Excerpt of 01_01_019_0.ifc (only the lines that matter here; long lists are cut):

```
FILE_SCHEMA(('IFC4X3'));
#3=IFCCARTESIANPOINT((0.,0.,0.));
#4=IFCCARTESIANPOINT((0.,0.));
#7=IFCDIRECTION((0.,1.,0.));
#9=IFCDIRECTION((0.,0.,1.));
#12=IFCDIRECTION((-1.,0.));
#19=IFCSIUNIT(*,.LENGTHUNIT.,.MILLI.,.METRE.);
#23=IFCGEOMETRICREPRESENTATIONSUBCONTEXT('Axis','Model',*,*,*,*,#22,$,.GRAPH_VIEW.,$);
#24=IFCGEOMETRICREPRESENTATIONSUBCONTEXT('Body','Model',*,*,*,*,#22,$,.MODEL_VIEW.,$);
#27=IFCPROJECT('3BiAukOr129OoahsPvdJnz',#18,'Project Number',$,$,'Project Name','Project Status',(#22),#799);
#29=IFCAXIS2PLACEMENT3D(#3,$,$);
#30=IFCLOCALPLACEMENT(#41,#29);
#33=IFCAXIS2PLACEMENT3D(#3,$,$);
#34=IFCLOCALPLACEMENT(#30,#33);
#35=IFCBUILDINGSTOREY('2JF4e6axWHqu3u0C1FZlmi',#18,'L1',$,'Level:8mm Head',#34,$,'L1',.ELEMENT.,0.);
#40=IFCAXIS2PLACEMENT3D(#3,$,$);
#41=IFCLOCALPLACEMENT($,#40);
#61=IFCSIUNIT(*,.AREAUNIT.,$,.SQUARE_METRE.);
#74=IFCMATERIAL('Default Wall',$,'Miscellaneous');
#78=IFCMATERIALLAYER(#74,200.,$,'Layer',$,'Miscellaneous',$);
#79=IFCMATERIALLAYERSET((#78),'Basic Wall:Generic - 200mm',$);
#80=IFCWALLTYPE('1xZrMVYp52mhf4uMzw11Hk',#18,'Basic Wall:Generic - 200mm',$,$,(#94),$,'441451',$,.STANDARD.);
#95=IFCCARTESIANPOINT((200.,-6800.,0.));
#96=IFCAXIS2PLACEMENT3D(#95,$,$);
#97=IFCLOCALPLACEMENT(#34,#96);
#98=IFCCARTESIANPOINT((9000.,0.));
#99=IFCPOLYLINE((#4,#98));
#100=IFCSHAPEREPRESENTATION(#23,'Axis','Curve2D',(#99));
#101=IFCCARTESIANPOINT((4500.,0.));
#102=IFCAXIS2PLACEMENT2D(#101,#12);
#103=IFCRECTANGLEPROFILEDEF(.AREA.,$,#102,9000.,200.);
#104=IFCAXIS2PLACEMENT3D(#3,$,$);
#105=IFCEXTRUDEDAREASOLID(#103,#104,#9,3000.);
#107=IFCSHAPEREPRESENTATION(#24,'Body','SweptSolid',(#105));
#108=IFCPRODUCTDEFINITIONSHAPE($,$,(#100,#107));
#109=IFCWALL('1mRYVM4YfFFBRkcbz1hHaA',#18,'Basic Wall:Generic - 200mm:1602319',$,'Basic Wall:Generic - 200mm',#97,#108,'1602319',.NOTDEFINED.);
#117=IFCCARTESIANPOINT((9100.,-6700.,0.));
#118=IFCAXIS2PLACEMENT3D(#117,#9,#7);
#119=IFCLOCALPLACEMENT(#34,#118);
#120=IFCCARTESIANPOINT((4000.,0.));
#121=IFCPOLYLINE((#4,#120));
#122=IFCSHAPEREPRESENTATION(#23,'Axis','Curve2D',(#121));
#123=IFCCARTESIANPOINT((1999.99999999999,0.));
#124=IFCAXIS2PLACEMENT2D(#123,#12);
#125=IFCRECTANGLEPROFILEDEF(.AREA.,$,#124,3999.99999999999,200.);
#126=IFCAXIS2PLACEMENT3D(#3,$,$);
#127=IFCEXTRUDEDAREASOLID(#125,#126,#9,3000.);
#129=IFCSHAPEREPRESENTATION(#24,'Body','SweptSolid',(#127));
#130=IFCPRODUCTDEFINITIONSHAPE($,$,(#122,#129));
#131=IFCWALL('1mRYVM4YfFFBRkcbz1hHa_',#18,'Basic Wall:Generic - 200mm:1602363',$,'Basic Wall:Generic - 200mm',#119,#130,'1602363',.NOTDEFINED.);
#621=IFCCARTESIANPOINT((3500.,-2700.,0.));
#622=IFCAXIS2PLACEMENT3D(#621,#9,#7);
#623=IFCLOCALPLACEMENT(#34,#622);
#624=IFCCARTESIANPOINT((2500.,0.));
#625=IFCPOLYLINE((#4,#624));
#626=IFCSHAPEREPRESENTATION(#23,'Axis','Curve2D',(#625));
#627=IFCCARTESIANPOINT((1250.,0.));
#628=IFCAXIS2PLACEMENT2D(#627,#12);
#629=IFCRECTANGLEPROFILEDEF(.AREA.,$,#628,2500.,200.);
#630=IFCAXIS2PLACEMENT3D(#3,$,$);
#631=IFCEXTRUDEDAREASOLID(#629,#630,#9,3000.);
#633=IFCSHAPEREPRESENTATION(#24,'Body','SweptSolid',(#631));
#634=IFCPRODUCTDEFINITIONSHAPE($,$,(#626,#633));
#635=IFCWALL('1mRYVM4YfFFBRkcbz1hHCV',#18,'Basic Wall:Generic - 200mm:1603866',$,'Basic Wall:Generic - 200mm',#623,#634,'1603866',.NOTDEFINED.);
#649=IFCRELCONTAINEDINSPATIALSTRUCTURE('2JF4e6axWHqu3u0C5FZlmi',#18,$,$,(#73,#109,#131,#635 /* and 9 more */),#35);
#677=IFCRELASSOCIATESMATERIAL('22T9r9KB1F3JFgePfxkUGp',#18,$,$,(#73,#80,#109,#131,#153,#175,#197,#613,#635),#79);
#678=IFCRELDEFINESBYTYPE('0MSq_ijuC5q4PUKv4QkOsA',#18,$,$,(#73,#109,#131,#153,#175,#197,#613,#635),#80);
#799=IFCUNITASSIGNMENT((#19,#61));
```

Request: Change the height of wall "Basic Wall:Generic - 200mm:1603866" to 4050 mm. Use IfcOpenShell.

```python
import ifcopenshell
import ifcopenshell.geom
import ifcopenshell.util.representation
import ifcopenshell.util.shape

model = ifcopenshell.open("01_01_019_0.ifc")
settings = ifcopenshell.geom.settings()


def volume(element):
    """Net volume in cubic metres, openings subtracted."""
    shape = ifcopenshell.geom.create_shape(settings, element)
    return ifcopenshell.util.shape.get_volume(shape.geometry)


wall = model.by_guid("1mRYVM4YfFFBRkcbz1hHCV")
before = volume(wall)

body = ifcopenshell.util.representation.get_representation(wall, "Model", "Body")
solid = body.Items[0]
old_height = solid.Depth
solid.Depth = 4050.0
after = volume(wall)

print(f"height {old_height:g} -> {solid.Depth:g}, volume {before:.3f} -> {after:.3f} m3")

model.write("01_01_019_0_rev.ifc")
```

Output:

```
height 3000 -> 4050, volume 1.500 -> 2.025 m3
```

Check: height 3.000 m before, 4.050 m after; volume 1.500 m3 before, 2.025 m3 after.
